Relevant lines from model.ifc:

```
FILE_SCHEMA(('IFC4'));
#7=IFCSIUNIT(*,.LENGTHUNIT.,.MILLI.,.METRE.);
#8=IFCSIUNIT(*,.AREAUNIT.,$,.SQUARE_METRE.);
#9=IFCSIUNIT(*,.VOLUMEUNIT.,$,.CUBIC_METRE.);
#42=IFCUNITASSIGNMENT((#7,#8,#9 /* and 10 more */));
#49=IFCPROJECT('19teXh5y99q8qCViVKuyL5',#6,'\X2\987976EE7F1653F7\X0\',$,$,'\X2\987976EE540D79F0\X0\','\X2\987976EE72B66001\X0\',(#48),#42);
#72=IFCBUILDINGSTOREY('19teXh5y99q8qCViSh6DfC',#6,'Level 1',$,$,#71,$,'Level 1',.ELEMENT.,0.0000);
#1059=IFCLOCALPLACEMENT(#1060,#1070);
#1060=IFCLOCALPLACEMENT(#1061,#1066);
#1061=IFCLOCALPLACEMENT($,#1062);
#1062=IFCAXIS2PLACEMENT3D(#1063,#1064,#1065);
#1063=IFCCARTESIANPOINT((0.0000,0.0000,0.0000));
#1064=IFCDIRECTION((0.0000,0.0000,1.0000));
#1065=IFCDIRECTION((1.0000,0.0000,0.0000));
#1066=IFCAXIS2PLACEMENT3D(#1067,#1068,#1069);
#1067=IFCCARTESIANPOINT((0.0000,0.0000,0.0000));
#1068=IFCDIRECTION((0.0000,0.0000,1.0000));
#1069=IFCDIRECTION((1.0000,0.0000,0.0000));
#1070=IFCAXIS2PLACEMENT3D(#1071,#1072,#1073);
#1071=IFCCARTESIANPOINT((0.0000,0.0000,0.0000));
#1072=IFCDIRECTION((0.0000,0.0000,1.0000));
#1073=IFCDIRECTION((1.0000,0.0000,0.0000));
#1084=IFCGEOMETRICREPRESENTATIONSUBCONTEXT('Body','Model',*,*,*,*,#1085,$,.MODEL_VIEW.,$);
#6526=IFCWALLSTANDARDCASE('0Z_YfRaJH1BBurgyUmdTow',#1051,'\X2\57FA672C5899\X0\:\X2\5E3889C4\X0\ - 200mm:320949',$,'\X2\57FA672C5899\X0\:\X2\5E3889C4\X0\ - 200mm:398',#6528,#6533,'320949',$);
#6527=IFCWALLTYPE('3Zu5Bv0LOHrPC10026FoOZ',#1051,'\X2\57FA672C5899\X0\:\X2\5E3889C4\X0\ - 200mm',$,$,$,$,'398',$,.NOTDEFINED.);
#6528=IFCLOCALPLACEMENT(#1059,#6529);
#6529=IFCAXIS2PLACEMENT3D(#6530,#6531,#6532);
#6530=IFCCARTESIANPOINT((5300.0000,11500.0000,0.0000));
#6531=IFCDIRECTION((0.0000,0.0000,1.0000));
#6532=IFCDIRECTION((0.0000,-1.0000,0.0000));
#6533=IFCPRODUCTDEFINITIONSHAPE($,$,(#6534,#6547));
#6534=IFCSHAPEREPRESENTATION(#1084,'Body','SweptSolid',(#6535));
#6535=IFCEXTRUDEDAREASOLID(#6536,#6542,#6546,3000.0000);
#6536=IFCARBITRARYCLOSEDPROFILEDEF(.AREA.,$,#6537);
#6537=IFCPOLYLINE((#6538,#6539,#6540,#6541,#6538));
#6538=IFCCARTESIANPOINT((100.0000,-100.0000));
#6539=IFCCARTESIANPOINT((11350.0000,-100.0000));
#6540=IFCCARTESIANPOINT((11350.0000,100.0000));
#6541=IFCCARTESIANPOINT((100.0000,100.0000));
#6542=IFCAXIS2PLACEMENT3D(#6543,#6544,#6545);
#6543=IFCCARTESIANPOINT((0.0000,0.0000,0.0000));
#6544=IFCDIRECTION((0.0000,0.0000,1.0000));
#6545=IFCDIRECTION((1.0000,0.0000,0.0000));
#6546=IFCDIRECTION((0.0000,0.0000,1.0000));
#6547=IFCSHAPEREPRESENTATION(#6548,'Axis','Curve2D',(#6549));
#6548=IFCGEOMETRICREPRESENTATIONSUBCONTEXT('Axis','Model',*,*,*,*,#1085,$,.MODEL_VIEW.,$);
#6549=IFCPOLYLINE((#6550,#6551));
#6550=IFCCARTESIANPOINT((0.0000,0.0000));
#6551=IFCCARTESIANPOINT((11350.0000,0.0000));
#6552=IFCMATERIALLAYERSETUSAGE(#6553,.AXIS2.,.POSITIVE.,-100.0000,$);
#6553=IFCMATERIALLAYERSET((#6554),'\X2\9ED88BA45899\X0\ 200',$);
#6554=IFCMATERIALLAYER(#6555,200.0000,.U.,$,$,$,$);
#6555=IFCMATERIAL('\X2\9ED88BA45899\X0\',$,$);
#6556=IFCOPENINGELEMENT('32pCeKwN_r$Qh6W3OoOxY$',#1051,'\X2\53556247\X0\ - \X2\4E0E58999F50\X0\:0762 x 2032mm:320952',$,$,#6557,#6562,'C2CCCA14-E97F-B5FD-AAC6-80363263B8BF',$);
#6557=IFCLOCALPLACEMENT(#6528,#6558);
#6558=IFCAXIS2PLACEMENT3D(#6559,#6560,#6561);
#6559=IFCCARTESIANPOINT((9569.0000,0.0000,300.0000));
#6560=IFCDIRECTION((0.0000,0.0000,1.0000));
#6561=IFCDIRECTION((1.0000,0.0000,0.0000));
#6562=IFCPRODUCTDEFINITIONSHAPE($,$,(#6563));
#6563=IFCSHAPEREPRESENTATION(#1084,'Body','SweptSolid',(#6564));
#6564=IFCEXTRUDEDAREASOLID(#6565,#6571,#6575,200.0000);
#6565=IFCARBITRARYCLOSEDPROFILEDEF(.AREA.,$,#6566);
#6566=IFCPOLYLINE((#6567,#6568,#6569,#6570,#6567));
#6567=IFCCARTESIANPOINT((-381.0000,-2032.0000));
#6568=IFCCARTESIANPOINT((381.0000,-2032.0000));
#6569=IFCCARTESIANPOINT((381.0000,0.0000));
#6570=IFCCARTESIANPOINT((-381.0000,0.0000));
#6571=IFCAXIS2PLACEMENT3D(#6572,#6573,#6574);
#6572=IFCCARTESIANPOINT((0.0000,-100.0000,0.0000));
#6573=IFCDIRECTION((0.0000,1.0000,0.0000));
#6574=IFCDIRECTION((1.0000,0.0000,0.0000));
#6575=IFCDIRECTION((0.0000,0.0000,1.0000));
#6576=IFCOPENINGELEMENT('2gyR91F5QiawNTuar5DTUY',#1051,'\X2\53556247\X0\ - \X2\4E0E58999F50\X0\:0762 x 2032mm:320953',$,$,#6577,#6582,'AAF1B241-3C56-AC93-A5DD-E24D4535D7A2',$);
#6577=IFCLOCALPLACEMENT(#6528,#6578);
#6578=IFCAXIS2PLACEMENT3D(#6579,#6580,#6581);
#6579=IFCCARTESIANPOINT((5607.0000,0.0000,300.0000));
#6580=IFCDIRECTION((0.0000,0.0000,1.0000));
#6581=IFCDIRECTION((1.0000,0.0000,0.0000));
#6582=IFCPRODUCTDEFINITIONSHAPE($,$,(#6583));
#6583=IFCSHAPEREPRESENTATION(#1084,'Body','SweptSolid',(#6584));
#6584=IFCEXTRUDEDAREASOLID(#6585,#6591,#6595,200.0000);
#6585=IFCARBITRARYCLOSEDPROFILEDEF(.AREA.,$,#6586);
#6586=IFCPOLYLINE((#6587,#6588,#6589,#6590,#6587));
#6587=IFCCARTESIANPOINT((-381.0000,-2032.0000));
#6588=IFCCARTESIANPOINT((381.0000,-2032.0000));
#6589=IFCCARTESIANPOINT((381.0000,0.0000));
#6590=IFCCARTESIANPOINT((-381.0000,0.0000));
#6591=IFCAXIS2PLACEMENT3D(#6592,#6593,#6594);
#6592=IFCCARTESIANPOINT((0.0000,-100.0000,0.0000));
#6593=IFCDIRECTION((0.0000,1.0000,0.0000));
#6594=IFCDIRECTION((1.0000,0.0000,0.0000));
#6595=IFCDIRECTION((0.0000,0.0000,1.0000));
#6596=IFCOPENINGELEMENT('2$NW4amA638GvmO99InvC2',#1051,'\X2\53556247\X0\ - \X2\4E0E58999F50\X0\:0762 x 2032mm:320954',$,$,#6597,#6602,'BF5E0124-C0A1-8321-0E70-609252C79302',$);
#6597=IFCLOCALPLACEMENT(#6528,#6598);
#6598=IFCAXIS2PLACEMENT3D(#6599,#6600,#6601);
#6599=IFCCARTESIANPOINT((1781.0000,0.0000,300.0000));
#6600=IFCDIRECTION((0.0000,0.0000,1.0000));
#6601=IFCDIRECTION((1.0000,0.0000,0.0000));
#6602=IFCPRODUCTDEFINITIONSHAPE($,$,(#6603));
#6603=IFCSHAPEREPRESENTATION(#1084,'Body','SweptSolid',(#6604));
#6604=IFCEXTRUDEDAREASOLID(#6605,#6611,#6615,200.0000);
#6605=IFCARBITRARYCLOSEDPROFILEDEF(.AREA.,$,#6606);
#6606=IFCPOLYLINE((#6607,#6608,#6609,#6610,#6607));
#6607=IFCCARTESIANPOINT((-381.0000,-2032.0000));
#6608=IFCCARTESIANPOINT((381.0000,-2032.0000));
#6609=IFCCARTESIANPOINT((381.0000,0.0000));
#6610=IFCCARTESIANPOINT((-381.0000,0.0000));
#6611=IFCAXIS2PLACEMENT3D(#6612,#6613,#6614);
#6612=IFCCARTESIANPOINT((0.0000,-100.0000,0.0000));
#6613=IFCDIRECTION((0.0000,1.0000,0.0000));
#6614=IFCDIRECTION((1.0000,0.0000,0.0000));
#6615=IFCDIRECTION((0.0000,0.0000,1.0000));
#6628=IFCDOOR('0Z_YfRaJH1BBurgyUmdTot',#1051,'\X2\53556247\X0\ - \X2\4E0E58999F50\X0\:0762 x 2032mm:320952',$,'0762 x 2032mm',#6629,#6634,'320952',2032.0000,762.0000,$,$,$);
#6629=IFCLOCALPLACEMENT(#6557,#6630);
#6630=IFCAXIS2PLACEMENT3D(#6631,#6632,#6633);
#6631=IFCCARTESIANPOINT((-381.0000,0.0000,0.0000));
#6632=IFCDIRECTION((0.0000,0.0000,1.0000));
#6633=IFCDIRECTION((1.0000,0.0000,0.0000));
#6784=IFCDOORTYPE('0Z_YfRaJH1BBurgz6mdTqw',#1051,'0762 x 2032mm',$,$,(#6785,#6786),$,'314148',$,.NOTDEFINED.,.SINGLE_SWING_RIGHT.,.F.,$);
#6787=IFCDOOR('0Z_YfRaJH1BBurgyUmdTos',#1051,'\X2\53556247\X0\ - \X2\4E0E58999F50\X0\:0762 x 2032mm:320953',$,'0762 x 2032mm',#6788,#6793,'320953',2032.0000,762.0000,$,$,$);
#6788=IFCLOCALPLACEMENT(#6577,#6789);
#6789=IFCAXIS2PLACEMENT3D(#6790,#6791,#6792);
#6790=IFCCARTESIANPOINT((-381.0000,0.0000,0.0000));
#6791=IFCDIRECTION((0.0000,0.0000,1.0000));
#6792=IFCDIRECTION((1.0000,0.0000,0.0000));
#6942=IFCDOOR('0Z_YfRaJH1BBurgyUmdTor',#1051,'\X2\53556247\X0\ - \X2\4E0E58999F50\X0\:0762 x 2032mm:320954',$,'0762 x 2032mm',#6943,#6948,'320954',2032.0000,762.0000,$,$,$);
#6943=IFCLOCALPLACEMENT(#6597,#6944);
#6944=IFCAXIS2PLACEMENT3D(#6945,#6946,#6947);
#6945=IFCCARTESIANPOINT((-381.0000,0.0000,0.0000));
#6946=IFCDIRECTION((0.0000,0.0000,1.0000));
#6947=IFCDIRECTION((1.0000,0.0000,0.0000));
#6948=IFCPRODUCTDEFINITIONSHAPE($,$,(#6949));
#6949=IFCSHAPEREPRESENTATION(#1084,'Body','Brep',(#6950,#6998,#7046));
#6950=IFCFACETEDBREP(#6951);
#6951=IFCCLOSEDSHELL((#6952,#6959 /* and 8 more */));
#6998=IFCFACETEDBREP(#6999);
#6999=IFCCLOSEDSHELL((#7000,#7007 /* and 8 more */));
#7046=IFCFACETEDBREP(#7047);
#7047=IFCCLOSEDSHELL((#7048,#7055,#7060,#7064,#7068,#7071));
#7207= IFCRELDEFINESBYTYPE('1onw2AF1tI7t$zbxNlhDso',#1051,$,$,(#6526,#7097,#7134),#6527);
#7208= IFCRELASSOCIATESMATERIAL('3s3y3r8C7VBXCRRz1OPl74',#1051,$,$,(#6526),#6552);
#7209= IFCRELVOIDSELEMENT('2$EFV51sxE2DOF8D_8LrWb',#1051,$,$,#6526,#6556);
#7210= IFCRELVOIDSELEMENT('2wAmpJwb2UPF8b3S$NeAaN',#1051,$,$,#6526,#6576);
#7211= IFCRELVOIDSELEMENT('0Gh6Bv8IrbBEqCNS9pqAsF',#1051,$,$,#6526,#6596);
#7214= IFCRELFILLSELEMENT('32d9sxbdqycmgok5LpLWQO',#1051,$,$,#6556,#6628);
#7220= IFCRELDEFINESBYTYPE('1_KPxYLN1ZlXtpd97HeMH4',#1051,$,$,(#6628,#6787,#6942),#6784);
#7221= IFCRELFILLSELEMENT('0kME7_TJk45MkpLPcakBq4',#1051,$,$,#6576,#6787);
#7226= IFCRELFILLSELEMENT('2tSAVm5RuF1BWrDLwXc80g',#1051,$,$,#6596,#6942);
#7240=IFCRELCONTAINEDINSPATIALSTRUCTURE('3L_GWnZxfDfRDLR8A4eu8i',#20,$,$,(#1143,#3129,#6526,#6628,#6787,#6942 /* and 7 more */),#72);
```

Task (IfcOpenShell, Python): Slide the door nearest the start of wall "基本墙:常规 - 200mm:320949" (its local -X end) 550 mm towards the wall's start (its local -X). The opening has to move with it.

```python
import ifcopenshell
import ifcopenshell.api.geometry
import ifcopenshell.util.placement
import ifcopenshell.util.unit

model = ifcopenshell.open("model.ifc")
unit_scale = ifcopenshell.util.unit.calculate_unit_scale(model)

door = model.by_guid("0Z_YfRaJH1BBurgyUmdTor")
opening = door.FillsVoids[0].RelatingOpeningElement
wall = opening.VoidsElements[0].RelatingBuildingElement

wall_matrix = ifcopenshell.util.placement.get_local_placement(wall.ObjectPlacement)
shift = wall_matrix[:3, 0] * -0.55 / unit_scale
before = ifcopenshell.util.placement.get_local_placement(door.ObjectPlacement)[:3, 3].copy()

# The door is placed relative to its opening, so it follows when the opening moves.
matrix = ifcopenshell.util.placement.get_local_placement(opening.ObjectPlacement)
matrix[:3, 3] += shift
ifcopenshell.api.geometry.edit_object_placement(
    model, product=opening, matrix=matrix, is_si=False, should_transform_children=True
)

after = ifcopenshell.util.placement.get_local_placement(door.ObjectPlacement)[:3, 3]
print("door moved by", (after - before).round(3) + 0.0)

model.write("model_v2.ifc")
```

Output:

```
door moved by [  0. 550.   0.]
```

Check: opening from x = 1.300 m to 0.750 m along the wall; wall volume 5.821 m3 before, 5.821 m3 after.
